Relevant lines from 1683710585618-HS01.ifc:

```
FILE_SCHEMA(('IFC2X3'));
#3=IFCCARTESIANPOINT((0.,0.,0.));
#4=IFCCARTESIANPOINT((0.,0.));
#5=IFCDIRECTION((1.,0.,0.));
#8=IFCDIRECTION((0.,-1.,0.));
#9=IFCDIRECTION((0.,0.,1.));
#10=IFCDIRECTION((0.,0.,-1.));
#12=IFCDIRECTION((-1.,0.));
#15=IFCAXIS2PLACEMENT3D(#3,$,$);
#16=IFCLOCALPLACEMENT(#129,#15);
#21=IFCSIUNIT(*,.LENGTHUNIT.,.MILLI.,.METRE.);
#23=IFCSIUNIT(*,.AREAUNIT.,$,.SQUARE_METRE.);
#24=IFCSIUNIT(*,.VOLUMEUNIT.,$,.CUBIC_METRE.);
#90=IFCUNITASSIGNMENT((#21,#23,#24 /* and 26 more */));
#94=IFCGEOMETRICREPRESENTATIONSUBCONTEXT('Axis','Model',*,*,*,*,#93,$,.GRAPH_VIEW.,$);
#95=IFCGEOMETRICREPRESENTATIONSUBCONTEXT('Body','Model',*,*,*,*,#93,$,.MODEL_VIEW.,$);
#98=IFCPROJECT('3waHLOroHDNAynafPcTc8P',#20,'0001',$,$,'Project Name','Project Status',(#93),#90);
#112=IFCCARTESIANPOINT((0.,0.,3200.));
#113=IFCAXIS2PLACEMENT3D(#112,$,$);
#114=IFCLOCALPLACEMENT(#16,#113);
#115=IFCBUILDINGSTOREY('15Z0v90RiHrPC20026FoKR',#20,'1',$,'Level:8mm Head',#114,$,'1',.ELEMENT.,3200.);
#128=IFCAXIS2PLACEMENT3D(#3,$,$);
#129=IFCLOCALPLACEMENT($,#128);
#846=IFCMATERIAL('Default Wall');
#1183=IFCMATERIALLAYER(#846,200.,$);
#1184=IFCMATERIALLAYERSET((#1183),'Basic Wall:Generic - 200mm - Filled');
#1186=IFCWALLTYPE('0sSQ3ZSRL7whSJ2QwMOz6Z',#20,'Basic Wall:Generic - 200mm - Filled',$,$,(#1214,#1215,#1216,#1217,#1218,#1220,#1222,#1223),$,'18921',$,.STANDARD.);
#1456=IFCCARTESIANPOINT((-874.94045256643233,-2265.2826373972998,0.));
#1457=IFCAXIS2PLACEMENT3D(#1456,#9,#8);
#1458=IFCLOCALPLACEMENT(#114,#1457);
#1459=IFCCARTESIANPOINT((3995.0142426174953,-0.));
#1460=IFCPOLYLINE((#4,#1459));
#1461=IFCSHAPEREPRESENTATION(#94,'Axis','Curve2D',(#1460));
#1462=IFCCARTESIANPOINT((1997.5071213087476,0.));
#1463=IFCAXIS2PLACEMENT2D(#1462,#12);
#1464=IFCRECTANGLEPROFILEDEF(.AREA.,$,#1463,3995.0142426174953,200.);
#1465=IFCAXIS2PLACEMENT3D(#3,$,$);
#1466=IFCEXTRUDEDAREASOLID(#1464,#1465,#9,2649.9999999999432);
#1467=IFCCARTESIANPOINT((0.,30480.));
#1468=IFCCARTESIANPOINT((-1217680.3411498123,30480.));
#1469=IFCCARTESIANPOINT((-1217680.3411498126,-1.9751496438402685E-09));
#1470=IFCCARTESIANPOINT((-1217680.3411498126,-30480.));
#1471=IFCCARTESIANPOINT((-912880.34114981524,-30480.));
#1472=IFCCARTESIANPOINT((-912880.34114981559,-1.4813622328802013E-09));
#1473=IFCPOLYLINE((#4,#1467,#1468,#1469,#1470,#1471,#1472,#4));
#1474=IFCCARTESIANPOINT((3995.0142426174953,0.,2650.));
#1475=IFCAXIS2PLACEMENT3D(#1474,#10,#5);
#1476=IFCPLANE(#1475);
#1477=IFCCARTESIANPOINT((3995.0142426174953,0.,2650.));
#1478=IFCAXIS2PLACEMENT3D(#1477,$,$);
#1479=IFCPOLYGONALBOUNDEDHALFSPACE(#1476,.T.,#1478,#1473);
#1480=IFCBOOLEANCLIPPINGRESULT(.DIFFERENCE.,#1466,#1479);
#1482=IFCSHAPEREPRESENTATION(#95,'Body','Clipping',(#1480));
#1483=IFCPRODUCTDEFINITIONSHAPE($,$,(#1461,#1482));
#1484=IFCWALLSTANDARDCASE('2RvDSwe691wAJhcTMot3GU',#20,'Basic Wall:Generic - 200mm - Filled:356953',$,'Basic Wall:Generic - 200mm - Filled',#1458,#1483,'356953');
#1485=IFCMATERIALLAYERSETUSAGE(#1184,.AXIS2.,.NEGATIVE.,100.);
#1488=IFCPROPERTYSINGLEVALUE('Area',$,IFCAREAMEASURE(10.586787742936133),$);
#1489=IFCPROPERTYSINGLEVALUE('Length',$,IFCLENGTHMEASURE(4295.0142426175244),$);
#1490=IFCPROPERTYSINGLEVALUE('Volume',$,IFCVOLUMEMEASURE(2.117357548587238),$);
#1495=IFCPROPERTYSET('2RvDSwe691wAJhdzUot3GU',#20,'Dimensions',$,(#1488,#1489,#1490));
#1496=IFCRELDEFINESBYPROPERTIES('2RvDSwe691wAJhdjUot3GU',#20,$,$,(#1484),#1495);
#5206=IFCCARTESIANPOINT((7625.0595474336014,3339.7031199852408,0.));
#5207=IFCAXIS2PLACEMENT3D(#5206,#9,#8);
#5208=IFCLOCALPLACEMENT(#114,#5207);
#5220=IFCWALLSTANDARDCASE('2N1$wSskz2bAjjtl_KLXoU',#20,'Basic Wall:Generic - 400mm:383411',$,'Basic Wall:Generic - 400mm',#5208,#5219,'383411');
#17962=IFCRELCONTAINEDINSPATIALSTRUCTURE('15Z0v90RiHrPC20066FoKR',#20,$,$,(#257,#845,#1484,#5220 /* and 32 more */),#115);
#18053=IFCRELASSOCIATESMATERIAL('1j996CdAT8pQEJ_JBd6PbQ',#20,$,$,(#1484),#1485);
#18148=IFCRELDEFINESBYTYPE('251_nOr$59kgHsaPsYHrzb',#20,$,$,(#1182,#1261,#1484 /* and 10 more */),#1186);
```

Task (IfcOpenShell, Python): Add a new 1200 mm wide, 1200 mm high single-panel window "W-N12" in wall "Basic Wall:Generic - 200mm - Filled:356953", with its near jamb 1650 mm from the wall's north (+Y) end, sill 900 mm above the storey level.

```python
import numpy as np
import ifcopenshell
import ifcopenshell.api.feature
import ifcopenshell.api.geometry
import ifcopenshell.api.pset
import ifcopenshell.api.root
import ifcopenshell.api.spatial
import ifcopenshell.api.type
import ifcopenshell.geom
import ifcopenshell.util.element
import ifcopenshell.util.placement
import ifcopenshell.util.representation
import ifcopenshell.util.shape
import ifcopenshell.util.unit

model = ifcopenshell.open("1683710585618-HS01.ifc")
unit_scale = ifcopenshell.util.unit.calculate_unit_scale(model)
area_scale = ifcopenshell.util.unit.calculate_unit_scale(model, "AREAUNIT")
volume_scale = ifcopenshell.util.unit.calculate_unit_scale(model, "VOLUMEUNIT")
settings = ifcopenshell.geom.settings()


def volume(element):
    """Net volume in cubic metres, openings subtracted."""
    shape = ifcopenshell.geom.create_shape(settings, element)
    return ifcopenshell.util.shape.get_volume(shape.geometry)


wall = model.by_guid("2RvDSwe691wAJhcTMot3GU")
storey = ifcopenshell.util.element.get_container(wall, ifc_class="IfcBuildingStorey")
context = ifcopenshell.util.representation.get_context(model, "Model", "Body", "MODEL_VIEW")
before = volume(wall)

width, height, from_end, sill = 1.2, 1.2, 1.65, 0.9  # metres

# The wall runs along its own X axis, and the end named is its -X end.
wall_shape = ifcopenshell.geom.create_shape(settings, wall)
x, y, z = ifcopenshell.util.shape.get_vertices(wall_shape.geometry).T
start = x.min() + from_end
face, thickness = float(y.min()), float(y.max() - y.min())
wall_matrix = ifcopenshell.util.placement.get_local_placement(wall.ObjectPlacement)
level = ifcopenshell.util.placement.get_local_placement(storey.ObjectPlacement)[2, 3]


def in_wall(x, y):
    """Placement at x, y metres in the wall's axes, at sill height."""
    matrix = wall_matrix.copy()
    matrix[:, 3] = wall_matrix @ np.array([x / unit_scale, y / unit_scale, 0.0, 1.0])
    matrix[2, 3] = level + sill / unit_scale
    return matrix


# Opening: a box that overshoots both wall faces by 50 mm.
opening = ifcopenshell.api.root.create_entity(model, ifc_class="IfcOpeningElement")
box = ifcopenshell.api.geometry.add_wall_representation(
    model, context=context, length=width, height=height, thickness=thickness + 0.1
)
ifcopenshell.api.geometry.assign_representation(model, product=opening, representation=box)
ifcopenshell.api.geometry.edit_object_placement(model, product=opening, matrix=in_wall(start, face - 0.05), is_si=False)
ifcopenshell.api.feature.add_feature(model, feature=opening, element=wall)

window = ifcopenshell.api.root.create_entity(model, ifc_class="IfcWindow", name="W-N12")
window.OverallWidth, window.OverallHeight = width / unit_scale, height / unit_scale
body = ifcopenshell.api.geometry.add_window_representation(
    model,
    context=context,
    overall_width=window.OverallWidth,
    overall_height=window.OverallHeight,
    partition_type="SINGLE_PANEL",
)
ifcopenshell.api.geometry.assign_representation(model, product=window, representation=body)
ifcopenshell.api.spatial.assign_container(model, products=[window], relating_structure=storey)
fills = ifcopenshell.api.feature.add_filling(model, opening=opening, element=window)
fills.OwnerHistory = window.OwnerHistory  # required in IFC2X3

# IFC2X3 keeps the operation on the window style.
style = ifcopenshell.api.root.create_entity(model, ifc_class="IfcWindowStyle", name="W-N12")
style.OperationType, style.ConstructionType = "SINGLE_PANEL", "NOTDEFINED"
style.ParameterTakesPrecedence = style.Sizeable = False
ifcopenshell.api.type.assign_type(model, related_objects=[window], relating_type=style)

# Centre the window in the wall's thickness.
ifcopenshell.api.geometry.edit_object_placement(model, product=window, matrix=in_wall(start, face), is_si=False)
window_shape = ifcopenshell.geom.create_shape(settings, window)
depth = ifcopenshell.util.shape.get_vertices(window_shape.geometry)[:, 1]
offset = face + thickness / 2 - (depth.min() + depth.max()) / 2
ifcopenshell.api.geometry.edit_object_placement(model, product=window, matrix=in_wall(start, offset), is_si=False)

after = volume(wall)

# Update the wall's stored quantities.
pset = model.by_id(ifcopenshell.util.element.get_pset(wall, "Dimensions", should_inherit=False)["id"])
ifcopenshell.api.pset.edit_pset(model, pset=pset, properties={
    "Area": model.create_entity("IfcAreaMeasure", after / thickness / area_scale),
    "Volume": model.create_entity("IfcVolumeMeasure", after / volume_scale),
})

print(f"wall volume {before:.3f} -> {after:.3f} m3")

model.write("1683710585618-HS01_edited.ifc")
```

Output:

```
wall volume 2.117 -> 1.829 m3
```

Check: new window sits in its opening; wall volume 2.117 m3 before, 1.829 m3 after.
